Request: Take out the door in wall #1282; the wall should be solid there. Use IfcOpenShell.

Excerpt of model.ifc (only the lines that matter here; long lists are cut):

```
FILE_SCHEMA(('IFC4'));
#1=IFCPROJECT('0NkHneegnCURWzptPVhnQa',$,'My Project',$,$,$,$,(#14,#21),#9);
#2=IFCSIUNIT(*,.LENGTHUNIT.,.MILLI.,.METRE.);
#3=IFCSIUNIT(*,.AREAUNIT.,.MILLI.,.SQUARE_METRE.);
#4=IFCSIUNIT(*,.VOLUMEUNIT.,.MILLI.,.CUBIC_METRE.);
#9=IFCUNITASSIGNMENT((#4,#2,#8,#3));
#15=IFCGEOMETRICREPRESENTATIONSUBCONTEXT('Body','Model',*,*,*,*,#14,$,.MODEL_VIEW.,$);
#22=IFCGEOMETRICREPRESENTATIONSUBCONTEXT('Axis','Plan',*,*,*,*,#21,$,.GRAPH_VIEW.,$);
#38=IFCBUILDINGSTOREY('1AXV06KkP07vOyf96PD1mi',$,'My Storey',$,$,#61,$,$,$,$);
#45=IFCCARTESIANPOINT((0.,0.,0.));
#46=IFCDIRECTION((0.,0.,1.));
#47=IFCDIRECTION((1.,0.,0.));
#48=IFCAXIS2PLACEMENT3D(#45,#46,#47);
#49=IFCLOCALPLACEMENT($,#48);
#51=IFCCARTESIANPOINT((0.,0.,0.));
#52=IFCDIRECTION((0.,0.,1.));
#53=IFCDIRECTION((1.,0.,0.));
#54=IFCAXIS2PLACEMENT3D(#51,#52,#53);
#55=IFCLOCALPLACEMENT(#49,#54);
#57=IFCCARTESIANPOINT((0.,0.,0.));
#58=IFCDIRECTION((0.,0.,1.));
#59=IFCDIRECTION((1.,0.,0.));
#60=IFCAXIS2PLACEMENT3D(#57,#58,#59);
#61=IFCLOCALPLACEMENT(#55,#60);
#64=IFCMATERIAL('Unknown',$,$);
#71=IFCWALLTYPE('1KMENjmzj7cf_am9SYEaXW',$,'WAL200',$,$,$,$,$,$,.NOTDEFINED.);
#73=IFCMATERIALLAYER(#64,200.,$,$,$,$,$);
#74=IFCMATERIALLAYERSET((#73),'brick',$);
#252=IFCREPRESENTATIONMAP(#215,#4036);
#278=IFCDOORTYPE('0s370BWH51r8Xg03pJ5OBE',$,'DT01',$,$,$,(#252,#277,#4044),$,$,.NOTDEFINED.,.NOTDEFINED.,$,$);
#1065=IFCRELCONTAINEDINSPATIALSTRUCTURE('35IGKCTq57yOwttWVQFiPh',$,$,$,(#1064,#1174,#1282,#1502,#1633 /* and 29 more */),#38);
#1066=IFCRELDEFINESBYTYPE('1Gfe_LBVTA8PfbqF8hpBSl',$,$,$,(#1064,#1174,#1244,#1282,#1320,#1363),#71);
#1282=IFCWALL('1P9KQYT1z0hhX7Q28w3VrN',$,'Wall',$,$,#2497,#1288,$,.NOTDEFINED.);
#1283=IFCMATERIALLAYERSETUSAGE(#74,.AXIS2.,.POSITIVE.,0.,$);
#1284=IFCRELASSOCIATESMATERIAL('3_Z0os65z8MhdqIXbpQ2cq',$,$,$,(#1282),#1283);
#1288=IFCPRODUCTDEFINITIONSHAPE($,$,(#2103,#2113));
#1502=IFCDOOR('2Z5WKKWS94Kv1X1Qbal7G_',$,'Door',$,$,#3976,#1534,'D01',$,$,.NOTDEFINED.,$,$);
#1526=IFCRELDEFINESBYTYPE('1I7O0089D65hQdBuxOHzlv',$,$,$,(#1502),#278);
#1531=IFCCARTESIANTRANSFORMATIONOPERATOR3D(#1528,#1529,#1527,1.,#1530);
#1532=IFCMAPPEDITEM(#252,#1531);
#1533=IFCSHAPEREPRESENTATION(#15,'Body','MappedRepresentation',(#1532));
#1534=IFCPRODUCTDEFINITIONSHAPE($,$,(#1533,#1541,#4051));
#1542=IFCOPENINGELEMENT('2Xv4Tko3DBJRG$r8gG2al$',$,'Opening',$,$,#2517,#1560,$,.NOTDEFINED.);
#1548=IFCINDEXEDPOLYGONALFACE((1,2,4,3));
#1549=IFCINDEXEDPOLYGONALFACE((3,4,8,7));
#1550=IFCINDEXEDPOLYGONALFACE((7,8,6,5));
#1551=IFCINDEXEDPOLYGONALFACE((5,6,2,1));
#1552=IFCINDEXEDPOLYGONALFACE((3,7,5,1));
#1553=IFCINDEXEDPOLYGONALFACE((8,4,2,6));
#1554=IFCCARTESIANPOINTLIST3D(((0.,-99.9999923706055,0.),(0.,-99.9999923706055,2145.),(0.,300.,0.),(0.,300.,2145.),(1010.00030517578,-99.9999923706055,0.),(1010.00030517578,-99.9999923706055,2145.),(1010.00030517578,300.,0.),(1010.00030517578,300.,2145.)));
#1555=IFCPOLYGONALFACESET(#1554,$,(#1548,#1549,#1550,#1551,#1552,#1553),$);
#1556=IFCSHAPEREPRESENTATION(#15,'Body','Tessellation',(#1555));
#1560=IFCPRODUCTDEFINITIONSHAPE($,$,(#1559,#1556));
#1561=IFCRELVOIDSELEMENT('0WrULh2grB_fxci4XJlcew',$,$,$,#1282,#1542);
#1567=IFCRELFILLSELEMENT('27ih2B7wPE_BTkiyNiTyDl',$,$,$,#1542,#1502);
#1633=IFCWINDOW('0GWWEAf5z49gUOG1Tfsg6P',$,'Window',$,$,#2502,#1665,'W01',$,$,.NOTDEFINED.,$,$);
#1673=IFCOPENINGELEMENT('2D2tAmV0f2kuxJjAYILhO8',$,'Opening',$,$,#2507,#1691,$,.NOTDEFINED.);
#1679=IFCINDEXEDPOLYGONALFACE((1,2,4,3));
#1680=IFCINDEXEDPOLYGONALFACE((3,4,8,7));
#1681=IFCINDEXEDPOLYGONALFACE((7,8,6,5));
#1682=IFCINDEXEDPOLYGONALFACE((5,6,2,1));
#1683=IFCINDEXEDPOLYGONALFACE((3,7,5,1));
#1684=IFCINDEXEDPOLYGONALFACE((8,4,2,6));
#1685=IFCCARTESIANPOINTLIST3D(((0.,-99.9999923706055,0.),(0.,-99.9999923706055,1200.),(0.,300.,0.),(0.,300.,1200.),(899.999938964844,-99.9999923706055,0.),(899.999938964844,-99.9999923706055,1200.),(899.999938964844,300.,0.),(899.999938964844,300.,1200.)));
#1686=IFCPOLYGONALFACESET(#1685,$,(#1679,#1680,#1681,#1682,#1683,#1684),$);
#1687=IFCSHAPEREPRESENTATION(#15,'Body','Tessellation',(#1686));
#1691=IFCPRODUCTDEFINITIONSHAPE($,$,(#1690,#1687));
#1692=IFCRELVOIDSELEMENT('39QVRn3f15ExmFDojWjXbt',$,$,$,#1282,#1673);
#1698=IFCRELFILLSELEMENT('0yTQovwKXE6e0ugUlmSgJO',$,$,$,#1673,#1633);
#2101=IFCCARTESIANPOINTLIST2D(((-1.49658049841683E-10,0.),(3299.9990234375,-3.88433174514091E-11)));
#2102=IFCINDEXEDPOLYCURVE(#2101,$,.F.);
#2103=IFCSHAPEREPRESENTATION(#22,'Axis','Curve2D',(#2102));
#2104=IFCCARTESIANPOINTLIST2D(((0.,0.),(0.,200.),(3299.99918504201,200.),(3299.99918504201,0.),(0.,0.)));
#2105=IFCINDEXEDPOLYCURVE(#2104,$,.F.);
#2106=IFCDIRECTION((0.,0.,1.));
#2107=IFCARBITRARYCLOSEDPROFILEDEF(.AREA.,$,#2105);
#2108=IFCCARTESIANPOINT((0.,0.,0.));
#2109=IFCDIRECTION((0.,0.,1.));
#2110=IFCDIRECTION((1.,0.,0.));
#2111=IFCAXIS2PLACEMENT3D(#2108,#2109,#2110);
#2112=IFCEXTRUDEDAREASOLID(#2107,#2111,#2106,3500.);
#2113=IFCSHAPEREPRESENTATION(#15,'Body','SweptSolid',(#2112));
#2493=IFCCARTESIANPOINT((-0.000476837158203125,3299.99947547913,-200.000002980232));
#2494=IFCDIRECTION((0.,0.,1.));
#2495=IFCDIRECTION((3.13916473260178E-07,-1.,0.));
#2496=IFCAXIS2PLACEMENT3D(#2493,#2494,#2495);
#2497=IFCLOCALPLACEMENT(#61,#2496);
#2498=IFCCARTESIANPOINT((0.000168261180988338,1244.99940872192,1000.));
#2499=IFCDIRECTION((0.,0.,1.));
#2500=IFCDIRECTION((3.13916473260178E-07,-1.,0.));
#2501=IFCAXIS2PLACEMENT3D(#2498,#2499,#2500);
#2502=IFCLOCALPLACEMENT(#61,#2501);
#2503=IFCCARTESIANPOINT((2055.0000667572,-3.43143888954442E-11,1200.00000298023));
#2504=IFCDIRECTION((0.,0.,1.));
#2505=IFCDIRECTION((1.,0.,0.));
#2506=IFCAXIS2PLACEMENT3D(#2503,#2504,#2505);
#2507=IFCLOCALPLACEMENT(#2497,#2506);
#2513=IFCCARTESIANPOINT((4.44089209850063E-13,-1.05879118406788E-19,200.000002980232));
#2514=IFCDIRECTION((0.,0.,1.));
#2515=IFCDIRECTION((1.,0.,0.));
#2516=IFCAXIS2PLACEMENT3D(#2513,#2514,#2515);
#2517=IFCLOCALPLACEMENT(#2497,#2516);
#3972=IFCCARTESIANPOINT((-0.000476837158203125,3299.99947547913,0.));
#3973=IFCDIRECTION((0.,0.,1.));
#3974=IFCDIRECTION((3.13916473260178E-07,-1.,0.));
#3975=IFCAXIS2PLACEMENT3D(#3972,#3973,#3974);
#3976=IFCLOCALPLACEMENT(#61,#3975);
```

```python
import ifcopenshell
import ifcopenshell.api.feature
import ifcopenshell.api.root
import ifcopenshell.geom
import ifcopenshell.util.shape

model = ifcopenshell.open("model.ifc")
settings = ifcopenshell.geom.settings()


def volume(element):
    """Net volume in cubic metres, openings subtracted."""
    shape = ifcopenshell.geom.create_shape(settings, element)
    return ifcopenshell.util.shape.get_volume(shape.geometry)


door = model.by_id(1502)
opening = door.FillsVoids[0].RelatingOpeningElement
wall = opening.VoidsElements[0].RelatingBuildingElement
before = volume(wall)

ifcopenshell.api.root.remove_product(model, product=door)
ifcopenshell.api.feature.remove_feature(model, feature=opening)

after = volume(wall)

print(f"wall volume {before:.3f} -> {after:.3f} m3")

model.write("model-out.ifc")
```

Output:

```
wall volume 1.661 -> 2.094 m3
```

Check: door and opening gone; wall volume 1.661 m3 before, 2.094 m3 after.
